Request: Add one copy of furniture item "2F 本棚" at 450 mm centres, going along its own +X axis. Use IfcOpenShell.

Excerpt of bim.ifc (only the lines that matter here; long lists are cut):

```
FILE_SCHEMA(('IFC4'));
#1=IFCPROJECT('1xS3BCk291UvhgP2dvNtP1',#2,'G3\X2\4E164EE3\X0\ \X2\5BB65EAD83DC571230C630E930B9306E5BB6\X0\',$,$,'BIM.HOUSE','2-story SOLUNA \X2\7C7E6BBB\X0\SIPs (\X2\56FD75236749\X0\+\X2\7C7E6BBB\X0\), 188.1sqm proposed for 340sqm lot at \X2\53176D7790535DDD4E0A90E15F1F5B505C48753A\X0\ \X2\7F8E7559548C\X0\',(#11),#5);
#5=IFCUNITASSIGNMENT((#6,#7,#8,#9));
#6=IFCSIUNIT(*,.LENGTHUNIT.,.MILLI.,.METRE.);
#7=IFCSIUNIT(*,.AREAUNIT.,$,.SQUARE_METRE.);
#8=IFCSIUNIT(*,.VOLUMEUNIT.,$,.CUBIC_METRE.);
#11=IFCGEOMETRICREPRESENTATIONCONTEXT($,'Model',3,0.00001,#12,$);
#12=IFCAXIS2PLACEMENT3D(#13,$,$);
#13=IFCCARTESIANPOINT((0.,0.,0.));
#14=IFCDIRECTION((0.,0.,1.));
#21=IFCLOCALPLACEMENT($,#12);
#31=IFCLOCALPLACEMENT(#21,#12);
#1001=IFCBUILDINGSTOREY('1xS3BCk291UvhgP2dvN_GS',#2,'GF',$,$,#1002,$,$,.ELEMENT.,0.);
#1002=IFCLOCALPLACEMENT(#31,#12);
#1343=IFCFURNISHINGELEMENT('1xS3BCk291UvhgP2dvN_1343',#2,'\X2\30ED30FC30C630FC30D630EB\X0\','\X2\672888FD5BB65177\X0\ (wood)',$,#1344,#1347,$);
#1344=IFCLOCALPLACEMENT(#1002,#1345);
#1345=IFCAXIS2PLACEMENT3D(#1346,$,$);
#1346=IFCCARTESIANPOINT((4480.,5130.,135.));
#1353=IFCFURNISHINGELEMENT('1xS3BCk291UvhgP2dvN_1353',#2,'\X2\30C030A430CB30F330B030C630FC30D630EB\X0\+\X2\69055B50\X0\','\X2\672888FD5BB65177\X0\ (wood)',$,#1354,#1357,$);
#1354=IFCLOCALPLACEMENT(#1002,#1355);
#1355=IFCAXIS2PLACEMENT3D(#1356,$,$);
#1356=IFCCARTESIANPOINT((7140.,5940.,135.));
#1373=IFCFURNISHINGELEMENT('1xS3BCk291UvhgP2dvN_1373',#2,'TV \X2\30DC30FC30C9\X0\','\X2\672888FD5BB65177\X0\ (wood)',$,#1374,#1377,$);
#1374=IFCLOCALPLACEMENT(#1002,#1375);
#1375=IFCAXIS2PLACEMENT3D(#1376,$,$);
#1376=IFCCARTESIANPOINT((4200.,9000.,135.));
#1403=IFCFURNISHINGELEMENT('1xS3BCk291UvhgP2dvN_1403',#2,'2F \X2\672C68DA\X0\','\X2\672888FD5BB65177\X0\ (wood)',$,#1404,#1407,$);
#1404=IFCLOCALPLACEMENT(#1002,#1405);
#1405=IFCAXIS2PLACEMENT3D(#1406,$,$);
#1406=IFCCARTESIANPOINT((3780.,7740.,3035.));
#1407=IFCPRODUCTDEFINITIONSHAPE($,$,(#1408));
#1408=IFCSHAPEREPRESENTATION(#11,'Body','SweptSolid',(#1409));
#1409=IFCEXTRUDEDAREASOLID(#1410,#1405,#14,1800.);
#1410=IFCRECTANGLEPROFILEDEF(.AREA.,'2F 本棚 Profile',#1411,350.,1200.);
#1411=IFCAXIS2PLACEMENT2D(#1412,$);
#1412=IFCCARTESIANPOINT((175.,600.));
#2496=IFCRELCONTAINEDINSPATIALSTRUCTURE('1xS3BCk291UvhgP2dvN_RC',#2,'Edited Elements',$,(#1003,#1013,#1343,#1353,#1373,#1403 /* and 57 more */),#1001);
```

```python
import ifcopenshell
import ifcopenshell.api.geometry
import ifcopenshell.api.root
import ifcopenshell.util.element
import ifcopenshell.util.placement

model = ifcopenshell.open("bim.ifc")


def reuse_history(source, copy):
    """copy_class also copies each property set's owner history, people and application; keep the originals."""
    for rel in copy.IsDefinedBy:
        if rel.is_a("IfcRelDefinesByProperties") and (history := rel.RelatingPropertyDefinition.OwnerHistory):
            rel.RelatingPropertyDefinition.OwnerHistory = source.OwnerHistory
            ifcopenshell.util.element.remove_deep2(model, history)


source = model.by_guid("1xS3BCk291UvhgP2dvN_1403")
base = ifcopenshell.util.placement.get_local_placement(source.ObjectPlacement)
step = base[:3, 0] * 450.0

for i in range(1, 2):
    copy = ifcopenshell.api.root.copy_class(model, product=source)
    copy.Representation = ifcopenshell.util.element.copy_deep(
        model, source.Representation, exclude=["IfcGeometricRepresentationContext", "IfcRepresentationMap"]
    )
    reuse_history(source, copy)
    matrix = base.copy()
    matrix[:3, 3] += i * step
    print("added at", matrix[:3, 3].round(3) + 0.0)
    ifcopenshell.api.geometry.edit_object_placement(model, product=copy, matrix=matrix, is_si=False)

model.write("bim_updated.ifc")
```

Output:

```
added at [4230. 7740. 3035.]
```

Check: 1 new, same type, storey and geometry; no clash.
